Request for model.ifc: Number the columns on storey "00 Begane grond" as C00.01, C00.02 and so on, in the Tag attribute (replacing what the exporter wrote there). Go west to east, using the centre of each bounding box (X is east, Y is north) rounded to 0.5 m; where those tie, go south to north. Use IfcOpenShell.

First a look at what the model holds.

```python
import ifcopenshell
import ifcopenshell.util.element
import ifcopenshell.util.placement

model = ifcopenshell.open("model.ifc")
print(model.schema)
storey = next(s for s in model.by_type("IfcBuildingStorey") if s.Name == "00 Begane grond")
columns = [e for e in ifcopenshell.util.element.get_decomposition(storey) if e.is_a("IfcColumn")]
for e in sorted(columns, key=lambda e: e.id()):
    origin = ifcopenshell.util.placement.get_local_placement(e.ObjectPlacement)[:3, 3]
    print(e.id(), e.Tag, e.Name, origin.round(2) + 0.0, sep=" | ")
```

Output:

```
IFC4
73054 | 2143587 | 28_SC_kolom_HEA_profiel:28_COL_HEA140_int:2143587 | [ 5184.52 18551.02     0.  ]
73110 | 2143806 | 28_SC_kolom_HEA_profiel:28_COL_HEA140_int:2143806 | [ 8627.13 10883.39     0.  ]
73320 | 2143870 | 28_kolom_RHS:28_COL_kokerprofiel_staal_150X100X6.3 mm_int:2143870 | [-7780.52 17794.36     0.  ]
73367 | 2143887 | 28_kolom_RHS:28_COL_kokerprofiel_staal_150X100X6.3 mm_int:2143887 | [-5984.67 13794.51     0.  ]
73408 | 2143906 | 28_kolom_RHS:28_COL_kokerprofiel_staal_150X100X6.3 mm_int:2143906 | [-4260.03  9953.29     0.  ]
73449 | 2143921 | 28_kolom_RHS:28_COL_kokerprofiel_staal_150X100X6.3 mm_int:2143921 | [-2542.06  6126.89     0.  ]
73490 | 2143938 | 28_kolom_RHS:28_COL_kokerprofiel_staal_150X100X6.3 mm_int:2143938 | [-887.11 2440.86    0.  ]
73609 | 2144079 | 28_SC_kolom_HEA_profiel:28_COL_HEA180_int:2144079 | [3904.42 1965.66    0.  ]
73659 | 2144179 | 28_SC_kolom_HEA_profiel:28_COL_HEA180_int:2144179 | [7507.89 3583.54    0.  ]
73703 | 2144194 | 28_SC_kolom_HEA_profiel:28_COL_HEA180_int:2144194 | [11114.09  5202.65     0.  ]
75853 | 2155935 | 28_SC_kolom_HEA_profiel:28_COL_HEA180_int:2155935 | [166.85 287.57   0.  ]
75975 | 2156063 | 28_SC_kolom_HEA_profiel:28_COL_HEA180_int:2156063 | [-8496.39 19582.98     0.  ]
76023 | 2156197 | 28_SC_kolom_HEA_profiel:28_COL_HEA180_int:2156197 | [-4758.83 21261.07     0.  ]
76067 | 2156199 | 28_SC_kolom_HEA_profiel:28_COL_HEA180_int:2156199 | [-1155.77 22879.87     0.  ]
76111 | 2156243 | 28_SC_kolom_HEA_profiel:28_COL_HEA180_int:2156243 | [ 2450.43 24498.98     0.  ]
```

```python
import ifcopenshell
import ifcopenshell.geom
import ifcopenshell.util.element
import ifcopenshell.util.shape

model = ifcopenshell.open("model.ifc")
settings = ifcopenshell.geom.settings()
settings.set("use-world-coords", True)


def centre(element):
    shape = ifcopenshell.geom.create_shape(settings, element)
    return ifcopenshell.util.shape.get_bbox_centroid(shape.geometry)


storey = next(s for s in model.by_type("IfcBuildingStorey") if s.Name == "00 Begane grond")
columns = [e for e in ifcopenshell.util.element.get_decomposition(storey) if e.is_a("IfcColumn")]

# Insertion points can sit at a corner or the storey origin, so sort by the geometry (in metres).
centres = {e: centre(e) for e in columns}
columns.sort(key=lambda e: (round(centres[e][0] / 0.5), centres[e][1]))

for i, e in enumerate(columns, start=1):
    number = f"C00.{i:02d}"
    e.Tag = number
    print(e.id(), number)

model.write("model_updated.ifc")
```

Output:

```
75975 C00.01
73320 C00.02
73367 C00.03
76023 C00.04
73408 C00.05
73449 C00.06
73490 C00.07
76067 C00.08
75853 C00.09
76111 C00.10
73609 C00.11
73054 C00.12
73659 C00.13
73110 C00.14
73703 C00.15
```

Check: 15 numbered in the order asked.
